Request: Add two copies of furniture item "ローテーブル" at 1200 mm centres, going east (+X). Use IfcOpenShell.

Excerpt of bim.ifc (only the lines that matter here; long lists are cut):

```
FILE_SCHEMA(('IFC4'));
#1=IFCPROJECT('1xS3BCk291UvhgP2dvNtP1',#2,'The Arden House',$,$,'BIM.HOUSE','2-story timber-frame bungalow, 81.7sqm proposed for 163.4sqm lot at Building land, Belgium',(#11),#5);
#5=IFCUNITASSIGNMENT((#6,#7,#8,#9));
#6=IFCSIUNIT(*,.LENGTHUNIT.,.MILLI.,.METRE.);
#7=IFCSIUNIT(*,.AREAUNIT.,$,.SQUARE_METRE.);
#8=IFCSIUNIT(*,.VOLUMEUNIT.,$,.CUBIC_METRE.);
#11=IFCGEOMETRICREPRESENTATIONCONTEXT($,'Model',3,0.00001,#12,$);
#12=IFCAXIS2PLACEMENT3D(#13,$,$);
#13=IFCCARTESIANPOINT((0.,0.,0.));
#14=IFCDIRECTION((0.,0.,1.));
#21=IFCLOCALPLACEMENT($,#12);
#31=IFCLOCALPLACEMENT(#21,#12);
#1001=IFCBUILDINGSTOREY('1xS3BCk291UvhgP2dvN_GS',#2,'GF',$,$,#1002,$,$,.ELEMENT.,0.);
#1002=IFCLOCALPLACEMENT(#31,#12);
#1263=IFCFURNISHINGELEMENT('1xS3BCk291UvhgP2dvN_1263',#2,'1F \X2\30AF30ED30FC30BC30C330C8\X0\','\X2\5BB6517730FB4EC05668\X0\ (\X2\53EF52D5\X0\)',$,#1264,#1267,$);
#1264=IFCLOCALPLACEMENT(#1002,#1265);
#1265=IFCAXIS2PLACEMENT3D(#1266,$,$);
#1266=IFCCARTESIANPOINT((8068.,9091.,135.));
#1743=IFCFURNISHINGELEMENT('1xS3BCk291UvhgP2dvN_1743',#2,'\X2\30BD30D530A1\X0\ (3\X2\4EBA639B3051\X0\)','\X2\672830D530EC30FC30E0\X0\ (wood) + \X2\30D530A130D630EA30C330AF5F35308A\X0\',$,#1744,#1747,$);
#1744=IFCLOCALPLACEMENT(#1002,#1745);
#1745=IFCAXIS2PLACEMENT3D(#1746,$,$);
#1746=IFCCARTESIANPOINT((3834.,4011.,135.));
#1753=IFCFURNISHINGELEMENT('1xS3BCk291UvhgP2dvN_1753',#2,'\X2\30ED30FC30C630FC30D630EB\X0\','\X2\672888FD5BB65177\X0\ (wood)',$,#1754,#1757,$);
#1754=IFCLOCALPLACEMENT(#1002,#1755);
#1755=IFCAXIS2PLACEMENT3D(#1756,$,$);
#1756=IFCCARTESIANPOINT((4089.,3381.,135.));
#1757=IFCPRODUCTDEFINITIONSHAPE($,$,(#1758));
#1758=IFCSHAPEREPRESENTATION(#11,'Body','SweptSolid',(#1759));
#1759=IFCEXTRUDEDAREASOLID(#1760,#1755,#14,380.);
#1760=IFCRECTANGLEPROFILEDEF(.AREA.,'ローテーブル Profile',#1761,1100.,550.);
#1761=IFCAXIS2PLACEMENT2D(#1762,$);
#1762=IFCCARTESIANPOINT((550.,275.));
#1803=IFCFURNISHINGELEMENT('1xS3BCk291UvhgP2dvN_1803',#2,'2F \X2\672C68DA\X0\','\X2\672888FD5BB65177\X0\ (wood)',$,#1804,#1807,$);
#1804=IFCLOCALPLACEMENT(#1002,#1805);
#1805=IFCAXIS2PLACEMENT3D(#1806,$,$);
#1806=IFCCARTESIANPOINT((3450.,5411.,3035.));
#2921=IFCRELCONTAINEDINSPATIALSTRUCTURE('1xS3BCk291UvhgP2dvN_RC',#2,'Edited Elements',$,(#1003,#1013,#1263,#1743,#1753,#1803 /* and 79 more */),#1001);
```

```python
import numpy as np
import ifcopenshell
import ifcopenshell.api.geometry
import ifcopenshell.api.root
import ifcopenshell.util.element
import ifcopenshell.util.placement
import ifcopenshell.util.unit

model = ifcopenshell.open("bim.ifc")
unit_scale = ifcopenshell.util.unit.calculate_unit_scale(model)


def reuse_history(source, copy):
    """copy_class also copies each property set's owner history, people and application; keep the originals."""
    for rel in copy.IsDefinedBy:
        if rel.is_a("IfcRelDefinesByProperties") and (history := rel.RelatingPropertyDefinition.OwnerHistory):
            rel.RelatingPropertyDefinition.OwnerHistory = source.OwnerHistory
            ifcopenshell.util.element.remove_deep2(model, history)


source = model.by_id(1753)
base = ifcopenshell.util.placement.get_local_placement(source.ObjectPlacement)
step = np.array([1.0, 0.0, 0.0]) * 1.2 / unit_scale

for i in range(1, 3):
    copy = ifcopenshell.api.root.copy_class(model, product=source)
    copy.Representation = ifcopenshell.util.element.copy_deep(
        model, source.Representation, exclude=["IfcGeometricRepresentationContext", "IfcRepresentationMap"]
    )
    reuse_history(source, copy)
    matrix = base.copy()
    matrix[:3, 3] += i * step
    print("added at", matrix[:3, 3].round(3) + 0.0)
    ifcopenshell.api.geometry.edit_object_placement(model, product=copy, matrix=matrix, is_si=False)

model.write("bim_updated.ifc")
```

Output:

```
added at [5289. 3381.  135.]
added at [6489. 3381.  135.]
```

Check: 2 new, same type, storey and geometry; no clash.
